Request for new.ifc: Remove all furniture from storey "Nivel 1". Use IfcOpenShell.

First a look at what the model holds.

```python
import ifcopenshell
import ifcopenshell.util.element

model = ifcopenshell.open("new.ifc")
print(model.schema)
storey = next(s for s in model.by_type("IfcBuildingStorey") if s.Name == "Nivel 1")
furniture = [e for e in ifcopenshell.util.element.get_decomposition(storey) if e.is_a("IfcFurnishingElement")]
seen = {}
for e in furniture:
    element_type = ifcopenshell.util.element.get_type(e)
    name = element_type.Name if element_type not in (None, e) else None
    seen[name] = seen.get(name, 0) + 1
for name, count in sorted(seen.items(), key=str):
    print(count, "x", name)
```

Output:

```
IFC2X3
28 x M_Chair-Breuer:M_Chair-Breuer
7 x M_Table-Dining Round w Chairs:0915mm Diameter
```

```python
import ifcopenshell
import ifcopenshell.api.root
import ifcopenshell.util.element

model = ifcopenshell.open("new.ifc")

storey = next(s for s in model.by_type("IfcBuildingStorey") if s.Name == "Nivel 1")
furniture = [e for e in ifcopenshell.util.element.get_decomposition(storey) if e.is_a("IfcFurnishingElement")]

for e in furniture:
    ifcopenshell.api.root.remove_product(model, product=e)
print(len(furniture), "removed")

model.write("new-out.ifc")
```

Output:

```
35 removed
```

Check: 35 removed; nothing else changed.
